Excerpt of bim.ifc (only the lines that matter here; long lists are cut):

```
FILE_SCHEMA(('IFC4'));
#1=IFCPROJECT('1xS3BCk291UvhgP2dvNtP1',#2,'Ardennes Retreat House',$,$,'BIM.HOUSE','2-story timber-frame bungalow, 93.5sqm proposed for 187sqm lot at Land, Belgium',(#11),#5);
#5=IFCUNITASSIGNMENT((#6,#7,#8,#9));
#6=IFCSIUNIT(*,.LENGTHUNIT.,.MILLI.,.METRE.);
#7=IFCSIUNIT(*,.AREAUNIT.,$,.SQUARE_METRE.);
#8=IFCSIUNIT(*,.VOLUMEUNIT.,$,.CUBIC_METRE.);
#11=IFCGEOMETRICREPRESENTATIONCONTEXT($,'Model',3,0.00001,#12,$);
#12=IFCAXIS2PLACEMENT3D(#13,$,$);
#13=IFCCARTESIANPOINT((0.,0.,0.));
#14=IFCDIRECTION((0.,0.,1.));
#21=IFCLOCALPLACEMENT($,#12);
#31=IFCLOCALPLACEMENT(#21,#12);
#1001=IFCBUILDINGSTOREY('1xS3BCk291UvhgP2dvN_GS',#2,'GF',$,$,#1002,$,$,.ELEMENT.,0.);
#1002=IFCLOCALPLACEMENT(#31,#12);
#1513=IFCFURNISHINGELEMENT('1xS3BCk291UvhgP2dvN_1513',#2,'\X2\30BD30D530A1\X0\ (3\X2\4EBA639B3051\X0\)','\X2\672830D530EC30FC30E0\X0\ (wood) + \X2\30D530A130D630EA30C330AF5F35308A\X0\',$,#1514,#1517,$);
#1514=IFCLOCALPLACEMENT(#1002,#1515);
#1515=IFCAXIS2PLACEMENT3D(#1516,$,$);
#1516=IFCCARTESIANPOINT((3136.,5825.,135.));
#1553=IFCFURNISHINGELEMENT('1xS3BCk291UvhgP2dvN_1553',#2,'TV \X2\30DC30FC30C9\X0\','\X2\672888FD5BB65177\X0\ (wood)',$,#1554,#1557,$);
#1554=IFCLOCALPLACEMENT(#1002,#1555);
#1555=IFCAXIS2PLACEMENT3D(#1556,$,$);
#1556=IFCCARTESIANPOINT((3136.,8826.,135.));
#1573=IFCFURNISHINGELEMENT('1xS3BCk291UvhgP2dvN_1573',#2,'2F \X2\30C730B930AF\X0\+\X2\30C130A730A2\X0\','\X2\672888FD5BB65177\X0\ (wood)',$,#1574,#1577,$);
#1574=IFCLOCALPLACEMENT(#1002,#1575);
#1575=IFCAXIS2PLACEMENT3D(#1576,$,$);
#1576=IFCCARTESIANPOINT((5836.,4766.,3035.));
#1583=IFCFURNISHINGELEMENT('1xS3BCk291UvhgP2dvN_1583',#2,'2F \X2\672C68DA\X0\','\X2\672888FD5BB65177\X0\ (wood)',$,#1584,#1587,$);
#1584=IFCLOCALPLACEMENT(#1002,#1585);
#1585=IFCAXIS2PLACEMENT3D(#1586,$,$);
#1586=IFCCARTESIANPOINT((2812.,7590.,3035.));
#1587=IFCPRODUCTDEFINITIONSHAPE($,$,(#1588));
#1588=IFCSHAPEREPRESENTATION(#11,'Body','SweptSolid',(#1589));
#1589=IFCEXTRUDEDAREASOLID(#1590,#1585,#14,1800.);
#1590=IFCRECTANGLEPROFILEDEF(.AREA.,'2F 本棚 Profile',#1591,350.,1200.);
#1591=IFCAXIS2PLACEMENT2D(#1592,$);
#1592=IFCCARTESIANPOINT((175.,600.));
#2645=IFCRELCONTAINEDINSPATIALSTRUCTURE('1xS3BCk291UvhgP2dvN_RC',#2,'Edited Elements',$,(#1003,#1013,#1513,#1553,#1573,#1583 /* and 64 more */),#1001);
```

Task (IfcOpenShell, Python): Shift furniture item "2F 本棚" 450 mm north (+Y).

```python
import ifcopenshell
import ifcopenshell.api.geometry
import ifcopenshell.util.placement
import ifcopenshell.util.unit

model = ifcopenshell.open("bim.ifc")
unit_scale = ifcopenshell.util.unit.calculate_unit_scale(model)

item = model.by_id(1583)
matrix = ifcopenshell.util.placement.get_local_placement(item.ObjectPlacement)
matrix[1, 3] += 0.45 / unit_scale
ifcopenshell.api.geometry.edit_object_placement(model, product=item, matrix=matrix, is_si=False)

print(ifcopenshell.util.placement.get_local_placement(item.ObjectPlacement).round(3) + 0.0)

model.write("bim_v2.ifc")
```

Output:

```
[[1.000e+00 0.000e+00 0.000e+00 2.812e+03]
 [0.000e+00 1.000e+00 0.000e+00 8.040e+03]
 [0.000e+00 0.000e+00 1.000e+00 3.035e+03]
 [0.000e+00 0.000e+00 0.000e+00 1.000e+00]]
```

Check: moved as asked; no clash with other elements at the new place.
